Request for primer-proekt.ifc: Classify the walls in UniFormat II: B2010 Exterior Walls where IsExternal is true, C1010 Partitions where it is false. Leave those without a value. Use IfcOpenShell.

First a look at what the model holds.

```python
import ifcopenshell
import ifcopenshell.util.element

model = ifcopenshell.open("primer-proekt.ifc")
print(model.schema)
print("classifications:", [c.Name for c in model.by_type("IfcClassification")])
values = [ifcopenshell.util.element.get_pset(e, "Pset_WallCommon", "IsExternal") for e in model.by_type("IfcWall")]
for value in (True, False, None):
    print("IsExternal", value, values.count(value))
```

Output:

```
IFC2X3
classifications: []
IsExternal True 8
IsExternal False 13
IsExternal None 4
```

```python
import ifcopenshell
import ifcopenshell.api.classification
import ifcopenshell.util.element

model = ifcopenshell.open("primer-proekt.ifc")

# IFC2X3 requires Source and Edition and has no link from the project to the system.
system = model.create_entity("IfcClassification", Source="ASTM", Edition="E1557", Name="UniFormat II")

walls = model.by_type("IfcWall")
external = {e: ifcopenshell.util.element.get_pset(e, "Pset_WallCommon", "IsExternal") for e in walls}
for flag, code, name in ((True, "B2010", "Exterior Walls"), (False, "C1010", "Partitions")):
    products = [e for e in walls if external[e] is flag]
    ifcopenshell.api.classification.add_reference(
        model, products=products, classification=system, identification=code, name=name
    )
    print(code, len(products))

model.write("primer-proekt_v2.ifc")
```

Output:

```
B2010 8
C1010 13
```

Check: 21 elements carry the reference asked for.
